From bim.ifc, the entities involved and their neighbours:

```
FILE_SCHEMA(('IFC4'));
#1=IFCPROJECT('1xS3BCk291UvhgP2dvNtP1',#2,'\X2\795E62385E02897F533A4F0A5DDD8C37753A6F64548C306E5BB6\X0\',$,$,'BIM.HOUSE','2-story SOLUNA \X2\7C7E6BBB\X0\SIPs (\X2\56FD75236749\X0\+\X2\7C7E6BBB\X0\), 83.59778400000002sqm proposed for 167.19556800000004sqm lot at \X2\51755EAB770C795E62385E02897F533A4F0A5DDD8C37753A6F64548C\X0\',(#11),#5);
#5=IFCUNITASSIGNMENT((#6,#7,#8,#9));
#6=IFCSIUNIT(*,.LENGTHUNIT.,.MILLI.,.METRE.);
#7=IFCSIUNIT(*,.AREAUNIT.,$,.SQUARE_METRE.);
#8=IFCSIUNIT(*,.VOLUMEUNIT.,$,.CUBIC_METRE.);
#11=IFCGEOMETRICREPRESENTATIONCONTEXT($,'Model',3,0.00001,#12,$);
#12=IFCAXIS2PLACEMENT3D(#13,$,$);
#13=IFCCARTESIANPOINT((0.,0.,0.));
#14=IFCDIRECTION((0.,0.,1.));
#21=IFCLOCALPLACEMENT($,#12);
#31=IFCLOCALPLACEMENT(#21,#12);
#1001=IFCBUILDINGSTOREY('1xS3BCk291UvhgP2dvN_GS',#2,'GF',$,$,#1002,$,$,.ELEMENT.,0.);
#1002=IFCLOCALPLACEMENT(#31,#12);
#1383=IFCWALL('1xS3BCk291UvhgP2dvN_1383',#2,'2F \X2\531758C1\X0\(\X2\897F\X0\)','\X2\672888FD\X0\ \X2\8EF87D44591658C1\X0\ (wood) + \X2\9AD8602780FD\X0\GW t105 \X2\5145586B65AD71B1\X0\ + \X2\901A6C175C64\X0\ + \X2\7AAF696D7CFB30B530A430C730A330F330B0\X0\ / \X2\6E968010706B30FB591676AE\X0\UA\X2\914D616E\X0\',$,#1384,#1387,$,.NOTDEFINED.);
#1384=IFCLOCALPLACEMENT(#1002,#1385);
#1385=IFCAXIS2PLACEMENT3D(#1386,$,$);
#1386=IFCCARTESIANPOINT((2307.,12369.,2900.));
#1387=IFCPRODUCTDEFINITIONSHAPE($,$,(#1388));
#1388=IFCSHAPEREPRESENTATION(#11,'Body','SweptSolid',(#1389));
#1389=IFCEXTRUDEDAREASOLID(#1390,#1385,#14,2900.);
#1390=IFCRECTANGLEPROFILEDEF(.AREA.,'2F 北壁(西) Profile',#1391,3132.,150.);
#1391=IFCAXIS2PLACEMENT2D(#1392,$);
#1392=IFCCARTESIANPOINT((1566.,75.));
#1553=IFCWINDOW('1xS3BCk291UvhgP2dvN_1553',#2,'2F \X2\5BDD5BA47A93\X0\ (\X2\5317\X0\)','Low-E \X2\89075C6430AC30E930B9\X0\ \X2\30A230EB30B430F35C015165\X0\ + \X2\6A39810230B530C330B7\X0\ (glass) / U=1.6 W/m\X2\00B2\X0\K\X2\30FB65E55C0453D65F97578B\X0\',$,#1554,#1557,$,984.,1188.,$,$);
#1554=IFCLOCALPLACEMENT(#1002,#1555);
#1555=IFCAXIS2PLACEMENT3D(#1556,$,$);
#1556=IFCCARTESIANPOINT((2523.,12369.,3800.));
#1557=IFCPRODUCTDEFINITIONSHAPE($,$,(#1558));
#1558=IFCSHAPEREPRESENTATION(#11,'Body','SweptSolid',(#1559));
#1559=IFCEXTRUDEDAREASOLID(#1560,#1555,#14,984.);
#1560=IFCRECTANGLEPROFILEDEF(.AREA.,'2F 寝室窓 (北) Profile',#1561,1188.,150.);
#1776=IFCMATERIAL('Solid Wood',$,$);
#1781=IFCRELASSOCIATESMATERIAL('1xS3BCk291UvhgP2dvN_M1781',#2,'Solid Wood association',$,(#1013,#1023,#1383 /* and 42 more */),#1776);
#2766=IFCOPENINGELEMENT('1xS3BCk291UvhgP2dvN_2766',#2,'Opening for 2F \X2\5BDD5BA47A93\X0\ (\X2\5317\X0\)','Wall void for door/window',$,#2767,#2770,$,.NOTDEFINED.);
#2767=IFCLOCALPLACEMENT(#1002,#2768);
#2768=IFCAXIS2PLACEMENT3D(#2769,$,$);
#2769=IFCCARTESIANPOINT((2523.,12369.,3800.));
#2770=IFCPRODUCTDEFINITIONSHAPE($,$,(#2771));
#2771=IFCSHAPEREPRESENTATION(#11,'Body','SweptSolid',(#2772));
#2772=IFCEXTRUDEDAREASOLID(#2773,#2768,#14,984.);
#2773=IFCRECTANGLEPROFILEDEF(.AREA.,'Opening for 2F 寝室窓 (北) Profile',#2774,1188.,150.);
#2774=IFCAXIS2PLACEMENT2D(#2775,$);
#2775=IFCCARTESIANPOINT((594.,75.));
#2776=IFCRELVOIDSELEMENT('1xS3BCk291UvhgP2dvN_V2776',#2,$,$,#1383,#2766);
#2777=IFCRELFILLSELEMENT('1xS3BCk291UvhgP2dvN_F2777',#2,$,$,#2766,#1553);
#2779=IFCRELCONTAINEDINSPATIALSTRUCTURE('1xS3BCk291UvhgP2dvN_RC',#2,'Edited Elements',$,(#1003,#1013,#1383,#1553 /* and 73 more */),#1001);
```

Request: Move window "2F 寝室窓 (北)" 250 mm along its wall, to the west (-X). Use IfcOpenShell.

```python
import ifcopenshell
import ifcopenshell.api.geometry
import ifcopenshell.util.placement
import ifcopenshell.util.unit

model = ifcopenshell.open("bim.ifc")
unit_scale = ifcopenshell.util.unit.calculate_unit_scale(model)

window = model.by_guid("1xS3BCk291UvhgP2dvN_1553")
opening = window.FillsVoids[0].RelatingOpeningElement
wall = opening.VoidsElements[0].RelatingBuildingElement

wall_matrix = ifcopenshell.util.placement.get_local_placement(wall.ObjectPlacement)
shift = wall_matrix[:3, 0] * -0.25 / unit_scale
before = ifcopenshell.util.placement.get_local_placement(window.ObjectPlacement)[:3, 3].copy()

# The window is not placed relative to its opening, so move both.
for product in (opening, window):
    matrix = ifcopenshell.util.placement.get_local_placement(product.ObjectPlacement)
    matrix[:3, 3] += shift
    ifcopenshell.api.geometry.edit_object_placement(model, product=product, matrix=matrix, is_si=False)

after = ifcopenshell.util.placement.get_local_placement(window.ObjectPlacement)[:3, 3]
print("window moved by", (after - before).round(3) + 0.0)

model.write("bim-out.ifc")
```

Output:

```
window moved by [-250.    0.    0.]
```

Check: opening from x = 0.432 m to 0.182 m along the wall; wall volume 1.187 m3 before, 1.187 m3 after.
